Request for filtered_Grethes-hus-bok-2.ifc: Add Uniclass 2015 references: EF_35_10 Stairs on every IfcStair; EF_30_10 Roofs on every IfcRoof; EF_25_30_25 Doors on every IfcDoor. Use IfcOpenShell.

First a look at what the model holds.

```python
import ifcopenshell

model = ifcopenshell.open("filtered_Grethes-hus-bok-2.ifc")
print(model.schema)
print("classifications:", [c.Name for c in model.by_type("IfcClassification")])
for ifc_class in ("IfcDoor", "IfcRoof", "IfcStair", "IfcWall", "IfcWindow"):
    print(ifc_class, len(model.by_type(ifc_class)))
```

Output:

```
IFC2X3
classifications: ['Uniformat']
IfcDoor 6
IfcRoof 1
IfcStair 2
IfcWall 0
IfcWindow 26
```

```python
import ifcopenshell
import ifcopenshell.api.classification

model = ifcopenshell.open("filtered_Grethes-hus-bok-2.ifc")

# IFC2X3 requires Source and Edition and has no link from the project to the system.
system = model.create_entity("IfcClassification", Source="NBS", Edition="2015", Name="Uniclass 2015")

codes = {
    "IfcStair": ("EF_35_10", "Stairs"),
    "IfcRoof": ("EF_30_10", "Roofs"),
    "IfcDoor": ("EF_25_30_25", "Doors"),
}
for ifc_class, (code, name) in codes.items():
    products = model.by_type(ifc_class)
    ifcopenshell.api.classification.add_reference(
        model, products=products, classification=system, identification=code, name=name
    )
    print(code, len(products))

model.write("filtered_Grethes-hus-bok-2-out.ifc")
```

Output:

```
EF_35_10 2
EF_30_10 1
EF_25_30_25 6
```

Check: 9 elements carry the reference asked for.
